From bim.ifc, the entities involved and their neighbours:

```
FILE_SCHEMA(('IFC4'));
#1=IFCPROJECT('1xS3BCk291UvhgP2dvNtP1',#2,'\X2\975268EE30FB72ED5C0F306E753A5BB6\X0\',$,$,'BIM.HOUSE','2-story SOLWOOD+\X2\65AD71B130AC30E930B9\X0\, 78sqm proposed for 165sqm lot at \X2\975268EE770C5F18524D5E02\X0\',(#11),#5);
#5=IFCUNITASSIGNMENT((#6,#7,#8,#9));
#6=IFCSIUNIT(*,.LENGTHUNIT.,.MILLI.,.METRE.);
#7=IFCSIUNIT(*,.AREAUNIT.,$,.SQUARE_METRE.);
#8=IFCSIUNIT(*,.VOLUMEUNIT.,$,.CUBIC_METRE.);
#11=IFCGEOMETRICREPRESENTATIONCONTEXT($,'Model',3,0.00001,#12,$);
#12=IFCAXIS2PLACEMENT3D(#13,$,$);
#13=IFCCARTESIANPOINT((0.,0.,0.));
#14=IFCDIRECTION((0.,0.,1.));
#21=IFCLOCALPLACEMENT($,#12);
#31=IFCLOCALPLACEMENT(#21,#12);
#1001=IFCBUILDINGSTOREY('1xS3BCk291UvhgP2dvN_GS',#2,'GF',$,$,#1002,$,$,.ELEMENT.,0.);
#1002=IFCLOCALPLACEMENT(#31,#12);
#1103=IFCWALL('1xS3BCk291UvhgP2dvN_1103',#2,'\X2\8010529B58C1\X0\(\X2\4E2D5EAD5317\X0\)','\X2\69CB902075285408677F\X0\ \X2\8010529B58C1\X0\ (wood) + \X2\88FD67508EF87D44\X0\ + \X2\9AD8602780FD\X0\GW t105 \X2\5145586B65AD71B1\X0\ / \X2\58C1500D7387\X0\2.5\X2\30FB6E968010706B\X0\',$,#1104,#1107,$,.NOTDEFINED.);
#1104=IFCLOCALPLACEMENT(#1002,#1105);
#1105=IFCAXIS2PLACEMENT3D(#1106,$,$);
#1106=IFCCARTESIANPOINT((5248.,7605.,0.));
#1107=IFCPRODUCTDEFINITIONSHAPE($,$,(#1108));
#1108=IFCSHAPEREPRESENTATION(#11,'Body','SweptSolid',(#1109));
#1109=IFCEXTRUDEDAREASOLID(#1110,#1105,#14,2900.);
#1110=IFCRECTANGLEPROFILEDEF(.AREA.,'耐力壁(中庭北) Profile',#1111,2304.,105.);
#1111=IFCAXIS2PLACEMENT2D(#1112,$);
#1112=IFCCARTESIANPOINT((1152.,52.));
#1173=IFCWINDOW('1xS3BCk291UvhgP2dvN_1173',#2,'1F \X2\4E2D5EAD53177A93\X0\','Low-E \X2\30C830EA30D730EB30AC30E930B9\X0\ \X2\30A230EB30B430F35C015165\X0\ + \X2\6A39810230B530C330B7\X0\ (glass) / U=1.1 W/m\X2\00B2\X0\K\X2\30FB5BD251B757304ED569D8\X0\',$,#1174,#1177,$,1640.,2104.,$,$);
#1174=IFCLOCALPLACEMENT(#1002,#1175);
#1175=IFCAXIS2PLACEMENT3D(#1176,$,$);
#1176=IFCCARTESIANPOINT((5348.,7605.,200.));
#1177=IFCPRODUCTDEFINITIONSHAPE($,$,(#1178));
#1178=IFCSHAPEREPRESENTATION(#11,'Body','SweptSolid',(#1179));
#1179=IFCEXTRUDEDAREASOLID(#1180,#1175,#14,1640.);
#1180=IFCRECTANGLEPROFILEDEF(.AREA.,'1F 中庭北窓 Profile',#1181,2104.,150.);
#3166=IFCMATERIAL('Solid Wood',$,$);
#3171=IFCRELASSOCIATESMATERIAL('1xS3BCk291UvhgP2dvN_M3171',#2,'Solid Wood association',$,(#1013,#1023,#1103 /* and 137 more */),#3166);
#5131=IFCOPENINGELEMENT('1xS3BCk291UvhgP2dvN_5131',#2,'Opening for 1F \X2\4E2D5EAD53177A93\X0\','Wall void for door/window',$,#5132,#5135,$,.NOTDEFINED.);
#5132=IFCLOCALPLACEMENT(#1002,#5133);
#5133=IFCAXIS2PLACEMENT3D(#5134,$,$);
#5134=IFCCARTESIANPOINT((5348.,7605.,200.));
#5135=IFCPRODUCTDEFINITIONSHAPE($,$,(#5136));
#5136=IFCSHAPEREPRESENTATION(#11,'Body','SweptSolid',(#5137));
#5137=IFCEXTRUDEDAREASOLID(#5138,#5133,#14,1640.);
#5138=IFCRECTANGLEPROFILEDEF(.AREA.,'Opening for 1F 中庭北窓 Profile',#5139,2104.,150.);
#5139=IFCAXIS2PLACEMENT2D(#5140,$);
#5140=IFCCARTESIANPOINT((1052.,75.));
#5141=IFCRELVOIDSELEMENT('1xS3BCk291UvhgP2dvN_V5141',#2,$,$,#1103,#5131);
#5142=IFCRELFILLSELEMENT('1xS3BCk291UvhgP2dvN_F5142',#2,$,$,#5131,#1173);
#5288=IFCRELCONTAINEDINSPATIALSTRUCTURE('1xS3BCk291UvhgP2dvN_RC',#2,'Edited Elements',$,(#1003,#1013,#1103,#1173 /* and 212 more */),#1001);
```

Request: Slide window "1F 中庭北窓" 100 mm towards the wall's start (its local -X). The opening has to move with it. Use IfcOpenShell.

```python
import ifcopenshell
import ifcopenshell.api.geometry
import ifcopenshell.util.placement
import ifcopenshell.util.unit

model = ifcopenshell.open("bim.ifc")
unit_scale = ifcopenshell.util.unit.calculate_unit_scale(model)

window = model.by_guid("1xS3BCk291UvhgP2dvN_1173")
opening = window.FillsVoids[0].RelatingOpeningElement
wall = opening.VoidsElements[0].RelatingBuildingElement

wall_matrix = ifcopenshell.util.placement.get_local_placement(wall.ObjectPlacement)
shift = wall_matrix[:3, 0] * -0.1 / unit_scale
before = ifcopenshell.util.placement.get_local_placement(window.ObjectPlacement)[:3, 3].copy()

# The window is not placed relative to its opening, so move both.
for product in (opening, window):
    matrix = ifcopenshell.util.placement.get_local_placement(product.ObjectPlacement)
    matrix[:3, 3] += shift
    ifcopenshell.api.geometry.edit_object_placement(model, product=product, matrix=matrix, is_si=False)

after = ifcopenshell.util.placement.get_local_placement(window.ObjectPlacement)[:3, 3]
print("window moved by", (after - before).round(3) + 0.0)

model.write("bim_updated.ifc")
```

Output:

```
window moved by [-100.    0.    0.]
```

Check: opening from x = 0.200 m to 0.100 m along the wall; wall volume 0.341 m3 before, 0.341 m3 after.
